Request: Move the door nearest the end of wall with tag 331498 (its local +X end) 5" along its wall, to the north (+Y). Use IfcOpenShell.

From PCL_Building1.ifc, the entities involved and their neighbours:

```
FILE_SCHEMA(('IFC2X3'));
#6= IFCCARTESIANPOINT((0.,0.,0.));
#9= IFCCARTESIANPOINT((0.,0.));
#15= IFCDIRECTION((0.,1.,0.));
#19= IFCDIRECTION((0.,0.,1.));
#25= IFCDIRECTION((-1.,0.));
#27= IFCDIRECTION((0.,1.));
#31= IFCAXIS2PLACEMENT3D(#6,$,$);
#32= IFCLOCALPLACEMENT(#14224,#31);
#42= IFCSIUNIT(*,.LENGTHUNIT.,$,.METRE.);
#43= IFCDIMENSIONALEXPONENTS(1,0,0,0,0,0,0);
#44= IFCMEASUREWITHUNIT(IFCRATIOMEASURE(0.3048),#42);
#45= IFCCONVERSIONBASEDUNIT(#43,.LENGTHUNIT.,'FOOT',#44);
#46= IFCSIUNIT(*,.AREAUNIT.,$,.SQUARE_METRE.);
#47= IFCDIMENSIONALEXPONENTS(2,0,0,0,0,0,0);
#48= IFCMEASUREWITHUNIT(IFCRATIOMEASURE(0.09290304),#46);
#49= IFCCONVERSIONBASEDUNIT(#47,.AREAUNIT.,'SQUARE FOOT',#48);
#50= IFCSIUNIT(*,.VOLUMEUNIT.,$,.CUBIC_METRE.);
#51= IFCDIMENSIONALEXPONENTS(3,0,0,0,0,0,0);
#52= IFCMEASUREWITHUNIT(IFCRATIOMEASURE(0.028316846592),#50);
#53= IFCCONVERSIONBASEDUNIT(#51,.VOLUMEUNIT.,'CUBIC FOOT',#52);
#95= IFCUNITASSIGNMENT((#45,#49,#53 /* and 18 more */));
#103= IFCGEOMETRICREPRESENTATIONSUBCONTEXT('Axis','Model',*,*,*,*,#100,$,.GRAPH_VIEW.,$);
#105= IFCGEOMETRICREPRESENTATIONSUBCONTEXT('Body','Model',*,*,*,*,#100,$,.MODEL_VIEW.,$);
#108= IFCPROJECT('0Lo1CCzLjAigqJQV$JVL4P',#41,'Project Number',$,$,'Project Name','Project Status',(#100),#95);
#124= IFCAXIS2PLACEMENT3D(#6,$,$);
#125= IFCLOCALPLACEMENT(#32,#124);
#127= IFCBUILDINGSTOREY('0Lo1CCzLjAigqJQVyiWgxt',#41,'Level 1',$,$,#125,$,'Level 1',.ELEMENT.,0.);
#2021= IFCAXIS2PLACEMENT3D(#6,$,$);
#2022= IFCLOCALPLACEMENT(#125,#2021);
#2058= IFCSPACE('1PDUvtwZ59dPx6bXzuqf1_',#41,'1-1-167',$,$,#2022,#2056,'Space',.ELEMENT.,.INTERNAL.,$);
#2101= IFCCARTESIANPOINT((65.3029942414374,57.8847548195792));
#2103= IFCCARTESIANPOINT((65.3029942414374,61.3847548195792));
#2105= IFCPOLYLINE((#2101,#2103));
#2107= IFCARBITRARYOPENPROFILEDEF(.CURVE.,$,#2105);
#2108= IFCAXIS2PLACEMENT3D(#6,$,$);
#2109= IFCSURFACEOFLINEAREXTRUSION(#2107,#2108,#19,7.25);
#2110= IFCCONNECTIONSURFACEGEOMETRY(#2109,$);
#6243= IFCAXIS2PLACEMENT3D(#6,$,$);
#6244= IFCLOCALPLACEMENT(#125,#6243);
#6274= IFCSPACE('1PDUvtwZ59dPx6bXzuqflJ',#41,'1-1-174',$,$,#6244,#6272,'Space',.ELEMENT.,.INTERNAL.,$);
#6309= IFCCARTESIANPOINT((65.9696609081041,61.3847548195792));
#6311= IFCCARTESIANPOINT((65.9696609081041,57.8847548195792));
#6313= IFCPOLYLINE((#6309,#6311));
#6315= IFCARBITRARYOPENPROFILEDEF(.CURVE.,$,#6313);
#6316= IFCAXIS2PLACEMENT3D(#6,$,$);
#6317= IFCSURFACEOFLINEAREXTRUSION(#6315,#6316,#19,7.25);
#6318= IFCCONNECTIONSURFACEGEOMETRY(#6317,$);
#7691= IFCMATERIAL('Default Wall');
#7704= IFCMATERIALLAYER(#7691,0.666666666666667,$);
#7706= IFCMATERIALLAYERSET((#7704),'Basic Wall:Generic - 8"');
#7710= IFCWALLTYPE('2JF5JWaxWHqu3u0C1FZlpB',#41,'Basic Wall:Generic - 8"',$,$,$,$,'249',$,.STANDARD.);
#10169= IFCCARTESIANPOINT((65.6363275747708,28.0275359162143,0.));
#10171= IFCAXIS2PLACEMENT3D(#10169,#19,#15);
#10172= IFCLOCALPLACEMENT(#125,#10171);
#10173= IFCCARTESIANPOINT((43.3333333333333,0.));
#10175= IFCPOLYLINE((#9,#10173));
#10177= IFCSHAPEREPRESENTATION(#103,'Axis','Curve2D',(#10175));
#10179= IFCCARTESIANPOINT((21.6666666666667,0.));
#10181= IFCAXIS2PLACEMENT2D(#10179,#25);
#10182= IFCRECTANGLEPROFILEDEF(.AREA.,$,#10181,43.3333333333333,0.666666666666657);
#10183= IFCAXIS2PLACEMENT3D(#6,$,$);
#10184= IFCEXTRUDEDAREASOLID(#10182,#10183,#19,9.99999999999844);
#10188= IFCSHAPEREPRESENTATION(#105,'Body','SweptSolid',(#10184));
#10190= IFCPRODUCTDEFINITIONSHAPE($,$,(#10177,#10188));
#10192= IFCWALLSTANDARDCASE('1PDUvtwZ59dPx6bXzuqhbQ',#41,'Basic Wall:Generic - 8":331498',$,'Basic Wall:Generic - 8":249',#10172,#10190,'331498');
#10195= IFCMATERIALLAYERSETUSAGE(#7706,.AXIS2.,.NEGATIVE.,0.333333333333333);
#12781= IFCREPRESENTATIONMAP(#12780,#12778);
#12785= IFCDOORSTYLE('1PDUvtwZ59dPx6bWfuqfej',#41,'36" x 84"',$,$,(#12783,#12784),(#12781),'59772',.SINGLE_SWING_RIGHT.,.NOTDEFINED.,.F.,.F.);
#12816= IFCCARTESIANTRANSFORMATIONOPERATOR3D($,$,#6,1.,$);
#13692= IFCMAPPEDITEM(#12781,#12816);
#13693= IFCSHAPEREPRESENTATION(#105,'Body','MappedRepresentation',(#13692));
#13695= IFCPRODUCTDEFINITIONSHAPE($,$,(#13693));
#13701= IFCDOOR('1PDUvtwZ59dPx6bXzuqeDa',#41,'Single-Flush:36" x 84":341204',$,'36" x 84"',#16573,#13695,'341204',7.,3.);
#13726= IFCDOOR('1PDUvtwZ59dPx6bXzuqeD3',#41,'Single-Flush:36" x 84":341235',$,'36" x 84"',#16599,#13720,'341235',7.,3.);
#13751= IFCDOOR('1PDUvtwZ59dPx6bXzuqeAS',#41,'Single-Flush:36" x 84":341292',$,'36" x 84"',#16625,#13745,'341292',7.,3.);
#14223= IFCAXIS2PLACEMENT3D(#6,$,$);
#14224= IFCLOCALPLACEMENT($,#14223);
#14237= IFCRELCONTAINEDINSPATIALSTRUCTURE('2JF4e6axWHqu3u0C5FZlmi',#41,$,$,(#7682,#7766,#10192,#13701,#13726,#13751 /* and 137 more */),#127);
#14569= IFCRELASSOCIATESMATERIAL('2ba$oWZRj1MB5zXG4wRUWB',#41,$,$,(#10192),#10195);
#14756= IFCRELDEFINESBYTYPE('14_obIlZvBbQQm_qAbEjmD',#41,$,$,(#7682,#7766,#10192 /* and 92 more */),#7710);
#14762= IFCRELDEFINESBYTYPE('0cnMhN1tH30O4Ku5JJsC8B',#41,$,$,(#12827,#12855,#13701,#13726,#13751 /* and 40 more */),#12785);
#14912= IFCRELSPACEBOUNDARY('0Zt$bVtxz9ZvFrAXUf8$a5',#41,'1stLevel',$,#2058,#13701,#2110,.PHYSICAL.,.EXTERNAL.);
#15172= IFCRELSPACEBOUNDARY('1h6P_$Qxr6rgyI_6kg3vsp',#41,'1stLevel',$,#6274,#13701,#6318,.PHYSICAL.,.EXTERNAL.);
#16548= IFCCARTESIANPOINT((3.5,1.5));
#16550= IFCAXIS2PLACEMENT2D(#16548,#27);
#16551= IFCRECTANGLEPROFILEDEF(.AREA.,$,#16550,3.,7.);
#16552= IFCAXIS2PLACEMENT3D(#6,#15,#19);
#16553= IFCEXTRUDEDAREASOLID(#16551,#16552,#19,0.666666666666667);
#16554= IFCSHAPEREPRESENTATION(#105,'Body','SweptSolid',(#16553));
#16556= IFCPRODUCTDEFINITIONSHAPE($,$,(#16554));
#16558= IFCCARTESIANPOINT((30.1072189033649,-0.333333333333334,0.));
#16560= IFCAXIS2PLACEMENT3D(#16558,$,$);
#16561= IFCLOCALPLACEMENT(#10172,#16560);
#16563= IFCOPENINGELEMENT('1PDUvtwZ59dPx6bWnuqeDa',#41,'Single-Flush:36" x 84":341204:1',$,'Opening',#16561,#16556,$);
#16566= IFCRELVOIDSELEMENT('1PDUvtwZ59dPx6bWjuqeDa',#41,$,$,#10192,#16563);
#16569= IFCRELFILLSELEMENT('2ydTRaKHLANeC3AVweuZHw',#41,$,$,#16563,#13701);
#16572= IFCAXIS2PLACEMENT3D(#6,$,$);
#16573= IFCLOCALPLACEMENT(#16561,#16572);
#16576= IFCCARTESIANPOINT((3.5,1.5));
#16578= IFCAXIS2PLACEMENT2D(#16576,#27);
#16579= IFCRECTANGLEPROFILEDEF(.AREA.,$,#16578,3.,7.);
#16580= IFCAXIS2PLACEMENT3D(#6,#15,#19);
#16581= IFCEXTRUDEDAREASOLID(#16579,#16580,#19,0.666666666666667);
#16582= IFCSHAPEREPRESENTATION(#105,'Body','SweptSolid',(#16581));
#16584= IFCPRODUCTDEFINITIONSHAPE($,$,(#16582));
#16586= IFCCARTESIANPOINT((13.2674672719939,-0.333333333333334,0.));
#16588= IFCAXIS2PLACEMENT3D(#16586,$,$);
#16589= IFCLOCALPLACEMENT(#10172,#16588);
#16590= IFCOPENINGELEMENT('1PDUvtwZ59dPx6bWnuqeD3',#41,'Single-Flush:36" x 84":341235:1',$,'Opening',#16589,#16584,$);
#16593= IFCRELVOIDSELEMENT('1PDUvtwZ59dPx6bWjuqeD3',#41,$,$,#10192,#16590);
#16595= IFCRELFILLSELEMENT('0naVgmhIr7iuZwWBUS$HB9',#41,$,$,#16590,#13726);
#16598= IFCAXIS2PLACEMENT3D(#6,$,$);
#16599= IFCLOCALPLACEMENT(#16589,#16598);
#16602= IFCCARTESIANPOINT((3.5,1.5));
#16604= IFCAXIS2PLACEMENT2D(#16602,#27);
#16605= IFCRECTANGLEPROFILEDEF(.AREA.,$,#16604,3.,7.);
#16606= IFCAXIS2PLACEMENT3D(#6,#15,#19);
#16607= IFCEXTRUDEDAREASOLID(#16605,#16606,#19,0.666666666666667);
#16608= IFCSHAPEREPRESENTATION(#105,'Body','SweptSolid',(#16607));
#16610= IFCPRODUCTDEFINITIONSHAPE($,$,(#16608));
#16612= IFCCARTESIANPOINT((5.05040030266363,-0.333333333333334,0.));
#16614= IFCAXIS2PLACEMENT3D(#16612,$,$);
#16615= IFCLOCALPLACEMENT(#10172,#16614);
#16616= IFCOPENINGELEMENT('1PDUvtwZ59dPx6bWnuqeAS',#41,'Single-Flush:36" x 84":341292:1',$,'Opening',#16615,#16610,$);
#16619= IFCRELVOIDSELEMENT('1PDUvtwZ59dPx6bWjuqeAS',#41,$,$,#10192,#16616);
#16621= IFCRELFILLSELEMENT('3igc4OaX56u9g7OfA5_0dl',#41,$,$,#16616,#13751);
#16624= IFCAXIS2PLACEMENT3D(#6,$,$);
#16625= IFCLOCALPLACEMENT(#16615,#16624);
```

```python
import numpy as np
import ifcopenshell
import ifcopenshell.api.geometry
import ifcopenshell.util.placement
import ifcopenshell.util.unit

model = ifcopenshell.open("PCL_Building1.ifc")
unit_scale = ifcopenshell.util.unit.calculate_unit_scale(model)

door = model.by_guid("1PDUvtwZ59dPx6bXzuqeDa")
opening = door.FillsVoids[0].RelatingOpeningElement
wall = opening.VoidsElements[0].RelatingBuildingElement

wall_matrix = ifcopenshell.util.placement.get_local_placement(wall.ObjectPlacement)
shift = wall_matrix[:3, 0] * 5 * 0.0254 / unit_scale
before = ifcopenshell.util.placement.get_local_placement(door.ObjectPlacement)[:3, 3].copy()

# The door is placed relative to its opening, so it follows when the opening moves.
matrix = ifcopenshell.util.placement.get_local_placement(opening.ObjectPlacement)
matrix[:3, 3] += shift
ifcopenshell.api.geometry.edit_object_placement(
    model, product=opening, matrix=matrix, is_si=False, should_transform_children=True
)

# Space boundary surfaces are stored in each space's coordinates; move them too.
for rel in door.ProvidesBoundaries:
    if not rel.ConnectionGeometry:
        continue
    surface = rel.ConnectionGeometry.SurfaceOnRelatingElement
    space_matrix = ifcopenshell.util.placement.get_local_placement(rel.RelatingSpace.ObjectPlacement)
    point = np.array(surface.Position.Location.Coordinates) + space_matrix[:3, :3].T @ shift
    surface.Position = model.createIfcAxis2Placement3D(
        model.createIfcCartesianPoint(point.tolist()), surface.Position.Axis, surface.Position.RefDirection
    )

after = ifcopenshell.util.placement.get_local_placement(door.ObjectPlacement)[:3, 3]
print("door moved by", (after - before).round(3) + 0.0)

model.write("PCL_Building1_updated.ifc")
```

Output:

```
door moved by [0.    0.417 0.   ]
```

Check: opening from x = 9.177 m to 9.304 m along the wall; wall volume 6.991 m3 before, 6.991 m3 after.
